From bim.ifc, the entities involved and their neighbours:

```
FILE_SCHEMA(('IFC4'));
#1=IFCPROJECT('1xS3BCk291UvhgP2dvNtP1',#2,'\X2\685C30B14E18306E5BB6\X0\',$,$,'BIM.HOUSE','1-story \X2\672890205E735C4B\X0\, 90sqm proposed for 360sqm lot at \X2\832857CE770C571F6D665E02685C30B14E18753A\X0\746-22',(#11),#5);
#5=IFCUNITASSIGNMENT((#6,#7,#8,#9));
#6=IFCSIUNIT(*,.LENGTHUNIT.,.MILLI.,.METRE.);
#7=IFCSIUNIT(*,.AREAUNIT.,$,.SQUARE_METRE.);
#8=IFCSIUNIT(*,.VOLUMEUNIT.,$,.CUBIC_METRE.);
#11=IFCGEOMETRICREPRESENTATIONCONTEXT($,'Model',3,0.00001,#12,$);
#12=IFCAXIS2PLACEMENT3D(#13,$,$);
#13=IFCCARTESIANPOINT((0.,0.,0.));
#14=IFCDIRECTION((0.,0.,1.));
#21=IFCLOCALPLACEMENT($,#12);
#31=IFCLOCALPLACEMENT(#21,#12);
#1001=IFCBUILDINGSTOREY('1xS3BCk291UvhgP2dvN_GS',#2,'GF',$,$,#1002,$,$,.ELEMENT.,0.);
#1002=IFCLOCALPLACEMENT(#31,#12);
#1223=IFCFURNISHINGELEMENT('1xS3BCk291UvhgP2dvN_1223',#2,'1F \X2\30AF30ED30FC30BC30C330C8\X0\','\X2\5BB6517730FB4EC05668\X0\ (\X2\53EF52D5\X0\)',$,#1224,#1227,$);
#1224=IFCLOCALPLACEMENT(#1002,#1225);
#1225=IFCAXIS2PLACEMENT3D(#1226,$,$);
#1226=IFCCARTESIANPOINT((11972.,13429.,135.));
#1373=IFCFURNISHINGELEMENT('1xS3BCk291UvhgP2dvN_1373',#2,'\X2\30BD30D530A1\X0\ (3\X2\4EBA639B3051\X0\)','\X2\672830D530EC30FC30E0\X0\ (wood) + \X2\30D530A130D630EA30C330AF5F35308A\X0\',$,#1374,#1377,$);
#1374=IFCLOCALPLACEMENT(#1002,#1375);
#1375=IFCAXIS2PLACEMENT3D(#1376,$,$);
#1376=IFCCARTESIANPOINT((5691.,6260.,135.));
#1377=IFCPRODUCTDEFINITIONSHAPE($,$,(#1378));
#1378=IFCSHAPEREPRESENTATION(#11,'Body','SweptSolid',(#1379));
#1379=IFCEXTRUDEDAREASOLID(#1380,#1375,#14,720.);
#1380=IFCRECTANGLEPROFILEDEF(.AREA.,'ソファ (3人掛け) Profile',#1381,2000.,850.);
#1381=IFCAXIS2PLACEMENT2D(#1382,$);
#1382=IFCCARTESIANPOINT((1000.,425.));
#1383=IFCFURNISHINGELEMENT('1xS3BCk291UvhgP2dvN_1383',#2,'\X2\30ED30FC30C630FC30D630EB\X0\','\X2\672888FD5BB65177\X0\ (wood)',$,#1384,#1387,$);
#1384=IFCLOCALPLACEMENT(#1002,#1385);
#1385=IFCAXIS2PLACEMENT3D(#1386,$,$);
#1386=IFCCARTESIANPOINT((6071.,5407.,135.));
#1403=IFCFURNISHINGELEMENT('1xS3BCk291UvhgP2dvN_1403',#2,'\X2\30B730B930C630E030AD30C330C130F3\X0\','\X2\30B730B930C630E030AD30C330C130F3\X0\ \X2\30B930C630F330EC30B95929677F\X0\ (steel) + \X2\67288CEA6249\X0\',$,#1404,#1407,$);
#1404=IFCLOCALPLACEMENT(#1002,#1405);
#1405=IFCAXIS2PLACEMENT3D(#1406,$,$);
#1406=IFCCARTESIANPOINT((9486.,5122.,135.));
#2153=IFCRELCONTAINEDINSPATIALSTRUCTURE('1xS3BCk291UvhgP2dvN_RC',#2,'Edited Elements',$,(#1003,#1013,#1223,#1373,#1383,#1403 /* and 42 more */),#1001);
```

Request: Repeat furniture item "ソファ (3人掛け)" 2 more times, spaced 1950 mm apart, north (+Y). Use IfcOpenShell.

```python
import numpy as np
import ifcopenshell
import ifcopenshell.api.geometry
import ifcopenshell.api.root
import ifcopenshell.util.element
import ifcopenshell.util.placement
import ifcopenshell.util.unit

model = ifcopenshell.open("bim.ifc")
unit_scale = ifcopenshell.util.unit.calculate_unit_scale(model)


def reuse_history(source, copy):
    """copy_class also copies each property set's owner history, people and application; keep the originals."""
    for rel in copy.IsDefinedBy:
        if rel.is_a("IfcRelDefinesByProperties") and (history := rel.RelatingPropertyDefinition.OwnerHistory):
            rel.RelatingPropertyDefinition.OwnerHistory = source.OwnerHistory
            ifcopenshell.util.element.remove_deep2(model, history)


source = model.by_guid("1xS3BCk291UvhgP2dvN_1373")
base = ifcopenshell.util.placement.get_local_placement(source.ObjectPlacement)
step = np.array([0.0, 1.0, 0.0]) * 1.95 / unit_scale

for i in range(1, 3):
    copy = ifcopenshell.api.root.copy_class(model, product=source)
    copy.Representation = ifcopenshell.util.element.copy_deep(
        model, source.Representation, exclude=["IfcGeometricRepresentationContext", "IfcRepresentationMap"]
    )
    reuse_history(source, copy)
    matrix = base.copy()
    matrix[:3, 3] += i * step
    print("added at", matrix[:3, 3].round(3) + 0.0)
    ifcopenshell.api.geometry.edit_object_placement(model, product=copy, matrix=matrix, is_si=False)

model.write("bim_updated.ifc")
```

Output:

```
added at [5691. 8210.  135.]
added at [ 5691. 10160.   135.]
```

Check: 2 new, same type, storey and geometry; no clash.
